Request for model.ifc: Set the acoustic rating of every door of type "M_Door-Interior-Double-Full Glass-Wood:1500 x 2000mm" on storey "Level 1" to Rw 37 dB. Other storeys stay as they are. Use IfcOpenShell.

First a look at what the model holds.

```python
import ifcopenshell
import ifcopenshell.util.element

model = ifcopenshell.open("model.ifc")
print(model.schema)
storey = next(s for s in model.by_type("IfcBuildingStorey") if s.Name == "Level 1")
doors = [e for e in ifcopenshell.util.element.get_decomposition(storey) if e.is_a("IfcDoor")]
seen = {}
for e in doors:
    element_type = ifcopenshell.util.element.get_type(e)
    key = (element_type.Name if element_type != e and element_type else None, ifcopenshell.util.element.get_pset(e, "Pset_DoorCommon", "AcousticRating"))
    seen[key] = seen.get(key, 0) + 1
for (name, value), count in sorted(seen.items(), key=str):
    print(count, "x", name, "|", value)
```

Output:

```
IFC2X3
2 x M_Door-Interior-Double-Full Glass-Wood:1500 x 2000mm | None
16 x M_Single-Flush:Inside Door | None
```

```python
import ifcopenshell
import ifcopenshell.api.pset
import ifcopenshell.util.element

model = ifcopenshell.open("model.ifc")

storey = next(s for s in model.by_type("IfcBuildingStorey") if s.Name == "Level 1")
doors = [e for e in ifcopenshell.util.element.get_decomposition(storey) if e.is_a("IfcDoor")]

count = 0
for e in doors:
    element_type = ifcopenshell.util.element.get_type(e)
    if element_type in (None, e) or element_type.Name != "M_Door-Interior-Double-Full Glass-Wood:1500 x 2000mm":
        continue
    # add_pset returns the element's existing set when there is one.
    pset = ifcopenshell.api.pset.add_pset(model, product=e, name="Pset_DoorCommon")
    ifcopenshell.api.pset.edit_pset(model, pset=pset, properties={"AcousticRating": "Rw 37 dB"})
    count += 1

print(count, "doors updated")

model.write("model_rev.ifc")
```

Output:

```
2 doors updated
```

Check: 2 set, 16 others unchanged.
